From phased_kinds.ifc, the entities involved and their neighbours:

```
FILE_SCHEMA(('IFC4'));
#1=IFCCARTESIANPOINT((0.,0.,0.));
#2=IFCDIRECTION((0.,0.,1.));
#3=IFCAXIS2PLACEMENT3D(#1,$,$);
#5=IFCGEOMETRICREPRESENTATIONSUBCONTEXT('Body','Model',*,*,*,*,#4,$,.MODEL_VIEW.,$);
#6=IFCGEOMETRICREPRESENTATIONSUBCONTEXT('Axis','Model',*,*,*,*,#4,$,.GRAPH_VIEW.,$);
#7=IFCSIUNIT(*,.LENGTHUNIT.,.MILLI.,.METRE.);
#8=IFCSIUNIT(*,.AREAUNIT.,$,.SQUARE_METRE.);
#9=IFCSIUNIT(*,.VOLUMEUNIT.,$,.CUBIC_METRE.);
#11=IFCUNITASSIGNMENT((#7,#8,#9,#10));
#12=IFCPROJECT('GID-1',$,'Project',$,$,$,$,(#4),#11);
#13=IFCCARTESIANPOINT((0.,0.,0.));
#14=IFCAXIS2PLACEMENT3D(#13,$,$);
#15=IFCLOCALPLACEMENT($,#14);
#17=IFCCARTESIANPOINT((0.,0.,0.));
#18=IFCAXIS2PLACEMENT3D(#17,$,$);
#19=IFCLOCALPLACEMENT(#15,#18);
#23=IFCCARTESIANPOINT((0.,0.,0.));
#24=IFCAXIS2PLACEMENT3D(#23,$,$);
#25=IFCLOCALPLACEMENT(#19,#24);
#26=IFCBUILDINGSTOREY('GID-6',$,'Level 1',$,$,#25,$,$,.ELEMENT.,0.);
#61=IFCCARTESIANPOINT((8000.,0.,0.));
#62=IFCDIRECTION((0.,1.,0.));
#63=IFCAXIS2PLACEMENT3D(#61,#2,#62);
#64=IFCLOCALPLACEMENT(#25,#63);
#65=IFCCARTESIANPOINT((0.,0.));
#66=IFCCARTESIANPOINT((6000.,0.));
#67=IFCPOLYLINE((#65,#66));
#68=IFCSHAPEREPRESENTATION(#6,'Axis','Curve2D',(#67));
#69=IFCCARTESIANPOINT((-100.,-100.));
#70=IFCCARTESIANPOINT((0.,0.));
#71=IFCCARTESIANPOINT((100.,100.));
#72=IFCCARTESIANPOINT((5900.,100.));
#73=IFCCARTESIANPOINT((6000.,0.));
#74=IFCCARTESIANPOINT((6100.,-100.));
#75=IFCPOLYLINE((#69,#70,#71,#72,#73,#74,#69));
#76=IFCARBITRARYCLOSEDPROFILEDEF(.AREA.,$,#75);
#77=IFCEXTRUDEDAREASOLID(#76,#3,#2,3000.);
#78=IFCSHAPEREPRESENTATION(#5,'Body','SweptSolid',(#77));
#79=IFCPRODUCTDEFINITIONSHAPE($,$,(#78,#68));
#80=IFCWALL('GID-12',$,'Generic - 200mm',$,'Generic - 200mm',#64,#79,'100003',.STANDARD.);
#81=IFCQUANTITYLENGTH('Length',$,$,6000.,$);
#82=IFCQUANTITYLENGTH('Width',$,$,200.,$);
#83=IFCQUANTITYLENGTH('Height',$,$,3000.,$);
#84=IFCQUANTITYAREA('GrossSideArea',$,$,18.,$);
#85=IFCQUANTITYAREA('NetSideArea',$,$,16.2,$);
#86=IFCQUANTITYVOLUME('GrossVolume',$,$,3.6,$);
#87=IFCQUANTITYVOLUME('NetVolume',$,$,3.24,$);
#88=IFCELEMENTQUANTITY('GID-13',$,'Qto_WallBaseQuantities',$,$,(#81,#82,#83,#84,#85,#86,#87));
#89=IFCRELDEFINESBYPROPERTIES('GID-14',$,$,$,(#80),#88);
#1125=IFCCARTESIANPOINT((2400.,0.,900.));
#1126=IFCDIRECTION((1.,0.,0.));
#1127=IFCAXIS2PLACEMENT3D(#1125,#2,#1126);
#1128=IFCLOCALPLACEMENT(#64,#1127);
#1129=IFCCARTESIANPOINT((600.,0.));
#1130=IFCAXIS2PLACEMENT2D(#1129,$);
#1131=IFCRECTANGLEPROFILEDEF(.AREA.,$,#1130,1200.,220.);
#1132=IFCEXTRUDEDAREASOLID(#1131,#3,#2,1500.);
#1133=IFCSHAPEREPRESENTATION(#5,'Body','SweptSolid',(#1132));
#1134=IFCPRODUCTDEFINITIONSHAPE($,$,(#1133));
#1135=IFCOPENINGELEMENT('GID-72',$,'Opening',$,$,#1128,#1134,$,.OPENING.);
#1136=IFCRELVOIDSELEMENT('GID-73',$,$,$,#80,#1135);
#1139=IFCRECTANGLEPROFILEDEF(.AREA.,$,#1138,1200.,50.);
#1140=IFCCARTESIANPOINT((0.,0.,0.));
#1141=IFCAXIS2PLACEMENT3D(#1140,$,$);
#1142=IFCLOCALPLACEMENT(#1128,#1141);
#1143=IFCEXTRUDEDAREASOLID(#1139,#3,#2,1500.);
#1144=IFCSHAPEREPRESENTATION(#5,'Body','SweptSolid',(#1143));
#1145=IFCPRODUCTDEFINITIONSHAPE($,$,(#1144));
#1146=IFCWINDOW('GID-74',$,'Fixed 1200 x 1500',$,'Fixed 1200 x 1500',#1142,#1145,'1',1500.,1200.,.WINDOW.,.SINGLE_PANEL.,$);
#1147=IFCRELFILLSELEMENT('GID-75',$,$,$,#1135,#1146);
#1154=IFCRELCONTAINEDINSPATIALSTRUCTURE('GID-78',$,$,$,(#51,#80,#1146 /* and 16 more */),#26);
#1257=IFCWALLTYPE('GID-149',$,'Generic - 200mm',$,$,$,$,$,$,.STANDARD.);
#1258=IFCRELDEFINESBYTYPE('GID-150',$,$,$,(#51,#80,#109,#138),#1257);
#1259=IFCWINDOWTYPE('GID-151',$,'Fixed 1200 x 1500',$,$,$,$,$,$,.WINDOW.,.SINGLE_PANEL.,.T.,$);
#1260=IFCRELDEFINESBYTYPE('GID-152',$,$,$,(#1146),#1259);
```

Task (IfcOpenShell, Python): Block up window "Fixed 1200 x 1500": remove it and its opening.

```python
import ifcopenshell
import ifcopenshell.api.feature
import ifcopenshell.api.pset
import ifcopenshell.api.root
import ifcopenshell.geom
import ifcopenshell.util.element
import ifcopenshell.util.shape
import ifcopenshell.util.unit

model = ifcopenshell.open("phased_kinds.ifc")
area_scale = ifcopenshell.util.unit.calculate_unit_scale(model, "AREAUNIT")
volume_scale = ifcopenshell.util.unit.calculate_unit_scale(model, "VOLUMEUNIT")
settings = ifcopenshell.geom.settings()


def volume(element):
    """Net volume in cubic metres, openings subtracted."""
    shape = ifcopenshell.geom.create_shape(settings, element)
    return ifcopenshell.util.shape.get_volume(shape.geometry)


window = model.by_guid("GID-74")
opening = window.FillsVoids[0].RelatingOpeningElement
wall = opening.VoidsElements[0].RelatingBuildingElement
before = volume(wall)

ifcopenshell.api.root.remove_product(model, product=window)
ifcopenshell.api.feature.remove_feature(model, feature=opening)

after = volume(wall)
thickness = 0.2  # wall thickness in metres

# Update the wall's stored quantities.
qto = model.by_id(ifcopenshell.util.element.get_pset(wall, "Qto_WallBaseQuantities", should_inherit=False)["id"])
ifcopenshell.api.pset.edit_qto(model, qto=qto, properties={
    "NetSideArea": after / thickness / area_scale,
    "NetVolume": after / volume_scale,
})

print(f"wall volume {before:.3f} -> {after:.3f} m3")

model.write("phased_kinds-out.ifc")
```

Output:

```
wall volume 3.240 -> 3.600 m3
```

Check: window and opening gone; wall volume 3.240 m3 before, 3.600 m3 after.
